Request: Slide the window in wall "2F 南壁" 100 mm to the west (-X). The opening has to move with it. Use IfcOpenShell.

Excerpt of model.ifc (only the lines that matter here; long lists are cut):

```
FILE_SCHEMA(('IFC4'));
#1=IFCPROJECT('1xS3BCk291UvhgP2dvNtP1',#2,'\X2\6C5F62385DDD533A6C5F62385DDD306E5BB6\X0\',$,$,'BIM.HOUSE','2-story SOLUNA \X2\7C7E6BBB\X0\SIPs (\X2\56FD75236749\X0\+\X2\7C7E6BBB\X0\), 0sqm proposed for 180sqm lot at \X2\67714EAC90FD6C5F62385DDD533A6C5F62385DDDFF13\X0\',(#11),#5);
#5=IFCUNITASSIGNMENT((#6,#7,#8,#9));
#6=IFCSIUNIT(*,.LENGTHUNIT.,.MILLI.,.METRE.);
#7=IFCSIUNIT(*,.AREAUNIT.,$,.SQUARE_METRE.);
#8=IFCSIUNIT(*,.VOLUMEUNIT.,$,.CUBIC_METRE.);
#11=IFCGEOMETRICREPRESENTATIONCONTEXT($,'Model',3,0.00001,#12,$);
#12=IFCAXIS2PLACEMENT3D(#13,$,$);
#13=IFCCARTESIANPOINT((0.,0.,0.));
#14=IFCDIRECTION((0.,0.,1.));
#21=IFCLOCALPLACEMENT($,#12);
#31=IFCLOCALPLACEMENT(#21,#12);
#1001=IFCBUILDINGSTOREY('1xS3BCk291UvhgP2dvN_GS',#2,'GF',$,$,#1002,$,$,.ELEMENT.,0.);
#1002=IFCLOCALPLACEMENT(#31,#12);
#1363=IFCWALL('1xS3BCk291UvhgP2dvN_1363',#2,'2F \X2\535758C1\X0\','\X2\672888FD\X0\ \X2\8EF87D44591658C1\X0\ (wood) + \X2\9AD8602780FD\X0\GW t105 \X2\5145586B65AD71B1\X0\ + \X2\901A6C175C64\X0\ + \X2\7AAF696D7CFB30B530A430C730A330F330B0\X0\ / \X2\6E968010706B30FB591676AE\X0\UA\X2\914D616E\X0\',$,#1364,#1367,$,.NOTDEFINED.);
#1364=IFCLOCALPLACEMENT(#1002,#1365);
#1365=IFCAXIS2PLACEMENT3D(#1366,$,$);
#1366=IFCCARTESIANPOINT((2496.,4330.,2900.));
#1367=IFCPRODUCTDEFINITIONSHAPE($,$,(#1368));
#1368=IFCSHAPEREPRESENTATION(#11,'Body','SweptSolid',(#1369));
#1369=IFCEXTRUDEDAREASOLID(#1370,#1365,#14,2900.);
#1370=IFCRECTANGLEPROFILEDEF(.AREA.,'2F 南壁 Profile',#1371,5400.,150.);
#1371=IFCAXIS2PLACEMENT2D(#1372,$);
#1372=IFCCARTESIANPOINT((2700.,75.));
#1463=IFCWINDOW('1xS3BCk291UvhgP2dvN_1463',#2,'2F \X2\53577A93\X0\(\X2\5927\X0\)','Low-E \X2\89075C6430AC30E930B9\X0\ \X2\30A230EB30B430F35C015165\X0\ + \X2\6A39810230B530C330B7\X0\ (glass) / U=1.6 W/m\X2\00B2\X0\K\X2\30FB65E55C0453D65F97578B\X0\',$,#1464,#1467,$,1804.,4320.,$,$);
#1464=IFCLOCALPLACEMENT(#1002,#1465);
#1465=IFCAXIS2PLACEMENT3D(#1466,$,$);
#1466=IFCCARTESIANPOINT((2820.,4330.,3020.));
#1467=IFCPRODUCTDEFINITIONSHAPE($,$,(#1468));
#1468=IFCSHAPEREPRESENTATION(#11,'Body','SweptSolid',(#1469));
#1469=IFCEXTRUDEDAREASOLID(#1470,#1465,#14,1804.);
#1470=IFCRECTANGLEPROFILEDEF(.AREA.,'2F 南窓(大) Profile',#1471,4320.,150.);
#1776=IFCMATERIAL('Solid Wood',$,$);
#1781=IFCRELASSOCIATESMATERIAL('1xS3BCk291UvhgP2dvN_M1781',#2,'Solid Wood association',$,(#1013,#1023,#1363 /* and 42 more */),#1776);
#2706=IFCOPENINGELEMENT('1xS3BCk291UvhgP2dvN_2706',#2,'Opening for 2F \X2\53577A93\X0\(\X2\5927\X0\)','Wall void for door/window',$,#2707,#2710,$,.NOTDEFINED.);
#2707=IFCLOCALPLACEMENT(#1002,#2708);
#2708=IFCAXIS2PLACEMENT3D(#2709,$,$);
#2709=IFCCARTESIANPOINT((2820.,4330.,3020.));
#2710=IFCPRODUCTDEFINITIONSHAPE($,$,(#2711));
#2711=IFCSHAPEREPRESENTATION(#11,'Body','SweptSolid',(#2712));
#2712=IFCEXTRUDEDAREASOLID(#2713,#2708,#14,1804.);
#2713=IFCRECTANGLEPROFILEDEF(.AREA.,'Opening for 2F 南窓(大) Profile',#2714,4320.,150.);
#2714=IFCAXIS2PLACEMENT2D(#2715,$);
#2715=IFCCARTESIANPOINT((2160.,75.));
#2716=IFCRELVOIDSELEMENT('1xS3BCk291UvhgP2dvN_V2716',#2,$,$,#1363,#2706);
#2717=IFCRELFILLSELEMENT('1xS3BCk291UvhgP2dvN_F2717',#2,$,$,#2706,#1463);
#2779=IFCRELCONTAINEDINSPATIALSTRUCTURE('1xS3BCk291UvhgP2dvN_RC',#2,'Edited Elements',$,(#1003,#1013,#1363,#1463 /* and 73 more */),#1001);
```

```python
import ifcopenshell
import ifcopenshell.api.geometry
import ifcopenshell.util.placement
import ifcopenshell.util.unit

model = ifcopenshell.open("model.ifc")
unit_scale = ifcopenshell.util.unit.calculate_unit_scale(model)

window = model.by_guid("1xS3BCk291UvhgP2dvN_1463")
opening = window.FillsVoids[0].RelatingOpeningElement
wall = opening.VoidsElements[0].RelatingBuildingElement

wall_matrix = ifcopenshell.util.placement.get_local_placement(wall.ObjectPlacement)
shift = wall_matrix[:3, 0] * -0.1 / unit_scale
before = ifcopenshell.util.placement.get_local_placement(window.ObjectPlacement)[:3, 3].copy()

# The window is not placed relative to its opening, so move both.
for product in (opening, window):
    matrix = ifcopenshell.util.placement.get_local_placement(product.ObjectPlacement)
    matrix[:3, 3] += shift
    ifcopenshell.api.geometry.edit_object_placement(model, product=product, matrix=matrix, is_si=False)

after = ifcopenshell.util.placement.get_local_placement(window.ObjectPlacement)[:3, 3]
print("window moved by", (after - before).round(3) + 0.0)

model.write("model-out.ifc")
```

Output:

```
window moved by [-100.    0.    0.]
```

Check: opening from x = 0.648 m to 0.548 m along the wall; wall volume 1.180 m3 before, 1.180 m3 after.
